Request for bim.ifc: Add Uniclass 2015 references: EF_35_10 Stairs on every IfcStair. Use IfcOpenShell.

First a look at what the model holds.

```python
import ifcopenshell

model = ifcopenshell.open("bim.ifc")
print(model.schema)
print("classifications:", [c.Name for c in model.by_type("IfcClassification")])
for ifc_class in ("IfcDoor", "IfcRoof", "IfcStair", "IfcWall", "IfcWindow"):
    print(ifc_class, len(model.by_type(ifc_class)))
```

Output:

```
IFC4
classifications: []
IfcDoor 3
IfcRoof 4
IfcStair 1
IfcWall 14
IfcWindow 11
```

```python
import ifcopenshell
import ifcopenshell.api.classification

model = ifcopenshell.open("bim.ifc")

system = ifcopenshell.api.classification.add_classification(model, classification="Uniclass 2015")

codes = {
    "IfcStair": ("EF_35_10", "Stairs"),
}
for ifc_class, (code, name) in codes.items():
    products = model.by_type(ifc_class)
    ifcopenshell.api.classification.add_reference(
        model, products=products, classification=system, identification=code, name=name
    )
    print(code, len(products))

model.write("bim-out.ifc")
```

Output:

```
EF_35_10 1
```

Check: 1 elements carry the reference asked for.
